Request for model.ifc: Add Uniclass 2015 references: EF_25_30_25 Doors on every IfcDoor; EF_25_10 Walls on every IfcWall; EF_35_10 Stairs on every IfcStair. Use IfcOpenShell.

First a look at what the model holds.

```python
import ifcopenshell

model = ifcopenshell.open("model.ifc")
print(model.schema)
print("classifications:", [c.Name for c in model.by_type("IfcClassification")])
for ifc_class in ("IfcDoor", "IfcRoof", "IfcStair", "IfcWall", "IfcWindow"):
    print(ifc_class, len(model.by_type(ifc_class)))
```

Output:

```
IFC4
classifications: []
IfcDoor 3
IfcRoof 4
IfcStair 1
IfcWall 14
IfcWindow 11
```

```python
import ifcopenshell
import ifcopenshell.api.classification

model = ifcopenshell.open("model.ifc")

system = ifcopenshell.api.classification.add_classification(model, classification="Uniclass 2015")

codes = {
    "IfcDoor": ("EF_25_30_25", "Doors"),
    "IfcWall": ("EF_25_10", "Walls"),
    "IfcStair": ("EF_35_10", "Stairs"),
}
for ifc_class, (code, name) in codes.items():
    products = model.by_type(ifc_class)
    ifcopenshell.api.classification.add_reference(
        model, products=products, classification=system, identification=code, name=name
    )
    print(code, len(products))

model.write("model_v2.ifc")
```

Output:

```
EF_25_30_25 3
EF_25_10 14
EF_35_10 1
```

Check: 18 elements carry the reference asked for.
